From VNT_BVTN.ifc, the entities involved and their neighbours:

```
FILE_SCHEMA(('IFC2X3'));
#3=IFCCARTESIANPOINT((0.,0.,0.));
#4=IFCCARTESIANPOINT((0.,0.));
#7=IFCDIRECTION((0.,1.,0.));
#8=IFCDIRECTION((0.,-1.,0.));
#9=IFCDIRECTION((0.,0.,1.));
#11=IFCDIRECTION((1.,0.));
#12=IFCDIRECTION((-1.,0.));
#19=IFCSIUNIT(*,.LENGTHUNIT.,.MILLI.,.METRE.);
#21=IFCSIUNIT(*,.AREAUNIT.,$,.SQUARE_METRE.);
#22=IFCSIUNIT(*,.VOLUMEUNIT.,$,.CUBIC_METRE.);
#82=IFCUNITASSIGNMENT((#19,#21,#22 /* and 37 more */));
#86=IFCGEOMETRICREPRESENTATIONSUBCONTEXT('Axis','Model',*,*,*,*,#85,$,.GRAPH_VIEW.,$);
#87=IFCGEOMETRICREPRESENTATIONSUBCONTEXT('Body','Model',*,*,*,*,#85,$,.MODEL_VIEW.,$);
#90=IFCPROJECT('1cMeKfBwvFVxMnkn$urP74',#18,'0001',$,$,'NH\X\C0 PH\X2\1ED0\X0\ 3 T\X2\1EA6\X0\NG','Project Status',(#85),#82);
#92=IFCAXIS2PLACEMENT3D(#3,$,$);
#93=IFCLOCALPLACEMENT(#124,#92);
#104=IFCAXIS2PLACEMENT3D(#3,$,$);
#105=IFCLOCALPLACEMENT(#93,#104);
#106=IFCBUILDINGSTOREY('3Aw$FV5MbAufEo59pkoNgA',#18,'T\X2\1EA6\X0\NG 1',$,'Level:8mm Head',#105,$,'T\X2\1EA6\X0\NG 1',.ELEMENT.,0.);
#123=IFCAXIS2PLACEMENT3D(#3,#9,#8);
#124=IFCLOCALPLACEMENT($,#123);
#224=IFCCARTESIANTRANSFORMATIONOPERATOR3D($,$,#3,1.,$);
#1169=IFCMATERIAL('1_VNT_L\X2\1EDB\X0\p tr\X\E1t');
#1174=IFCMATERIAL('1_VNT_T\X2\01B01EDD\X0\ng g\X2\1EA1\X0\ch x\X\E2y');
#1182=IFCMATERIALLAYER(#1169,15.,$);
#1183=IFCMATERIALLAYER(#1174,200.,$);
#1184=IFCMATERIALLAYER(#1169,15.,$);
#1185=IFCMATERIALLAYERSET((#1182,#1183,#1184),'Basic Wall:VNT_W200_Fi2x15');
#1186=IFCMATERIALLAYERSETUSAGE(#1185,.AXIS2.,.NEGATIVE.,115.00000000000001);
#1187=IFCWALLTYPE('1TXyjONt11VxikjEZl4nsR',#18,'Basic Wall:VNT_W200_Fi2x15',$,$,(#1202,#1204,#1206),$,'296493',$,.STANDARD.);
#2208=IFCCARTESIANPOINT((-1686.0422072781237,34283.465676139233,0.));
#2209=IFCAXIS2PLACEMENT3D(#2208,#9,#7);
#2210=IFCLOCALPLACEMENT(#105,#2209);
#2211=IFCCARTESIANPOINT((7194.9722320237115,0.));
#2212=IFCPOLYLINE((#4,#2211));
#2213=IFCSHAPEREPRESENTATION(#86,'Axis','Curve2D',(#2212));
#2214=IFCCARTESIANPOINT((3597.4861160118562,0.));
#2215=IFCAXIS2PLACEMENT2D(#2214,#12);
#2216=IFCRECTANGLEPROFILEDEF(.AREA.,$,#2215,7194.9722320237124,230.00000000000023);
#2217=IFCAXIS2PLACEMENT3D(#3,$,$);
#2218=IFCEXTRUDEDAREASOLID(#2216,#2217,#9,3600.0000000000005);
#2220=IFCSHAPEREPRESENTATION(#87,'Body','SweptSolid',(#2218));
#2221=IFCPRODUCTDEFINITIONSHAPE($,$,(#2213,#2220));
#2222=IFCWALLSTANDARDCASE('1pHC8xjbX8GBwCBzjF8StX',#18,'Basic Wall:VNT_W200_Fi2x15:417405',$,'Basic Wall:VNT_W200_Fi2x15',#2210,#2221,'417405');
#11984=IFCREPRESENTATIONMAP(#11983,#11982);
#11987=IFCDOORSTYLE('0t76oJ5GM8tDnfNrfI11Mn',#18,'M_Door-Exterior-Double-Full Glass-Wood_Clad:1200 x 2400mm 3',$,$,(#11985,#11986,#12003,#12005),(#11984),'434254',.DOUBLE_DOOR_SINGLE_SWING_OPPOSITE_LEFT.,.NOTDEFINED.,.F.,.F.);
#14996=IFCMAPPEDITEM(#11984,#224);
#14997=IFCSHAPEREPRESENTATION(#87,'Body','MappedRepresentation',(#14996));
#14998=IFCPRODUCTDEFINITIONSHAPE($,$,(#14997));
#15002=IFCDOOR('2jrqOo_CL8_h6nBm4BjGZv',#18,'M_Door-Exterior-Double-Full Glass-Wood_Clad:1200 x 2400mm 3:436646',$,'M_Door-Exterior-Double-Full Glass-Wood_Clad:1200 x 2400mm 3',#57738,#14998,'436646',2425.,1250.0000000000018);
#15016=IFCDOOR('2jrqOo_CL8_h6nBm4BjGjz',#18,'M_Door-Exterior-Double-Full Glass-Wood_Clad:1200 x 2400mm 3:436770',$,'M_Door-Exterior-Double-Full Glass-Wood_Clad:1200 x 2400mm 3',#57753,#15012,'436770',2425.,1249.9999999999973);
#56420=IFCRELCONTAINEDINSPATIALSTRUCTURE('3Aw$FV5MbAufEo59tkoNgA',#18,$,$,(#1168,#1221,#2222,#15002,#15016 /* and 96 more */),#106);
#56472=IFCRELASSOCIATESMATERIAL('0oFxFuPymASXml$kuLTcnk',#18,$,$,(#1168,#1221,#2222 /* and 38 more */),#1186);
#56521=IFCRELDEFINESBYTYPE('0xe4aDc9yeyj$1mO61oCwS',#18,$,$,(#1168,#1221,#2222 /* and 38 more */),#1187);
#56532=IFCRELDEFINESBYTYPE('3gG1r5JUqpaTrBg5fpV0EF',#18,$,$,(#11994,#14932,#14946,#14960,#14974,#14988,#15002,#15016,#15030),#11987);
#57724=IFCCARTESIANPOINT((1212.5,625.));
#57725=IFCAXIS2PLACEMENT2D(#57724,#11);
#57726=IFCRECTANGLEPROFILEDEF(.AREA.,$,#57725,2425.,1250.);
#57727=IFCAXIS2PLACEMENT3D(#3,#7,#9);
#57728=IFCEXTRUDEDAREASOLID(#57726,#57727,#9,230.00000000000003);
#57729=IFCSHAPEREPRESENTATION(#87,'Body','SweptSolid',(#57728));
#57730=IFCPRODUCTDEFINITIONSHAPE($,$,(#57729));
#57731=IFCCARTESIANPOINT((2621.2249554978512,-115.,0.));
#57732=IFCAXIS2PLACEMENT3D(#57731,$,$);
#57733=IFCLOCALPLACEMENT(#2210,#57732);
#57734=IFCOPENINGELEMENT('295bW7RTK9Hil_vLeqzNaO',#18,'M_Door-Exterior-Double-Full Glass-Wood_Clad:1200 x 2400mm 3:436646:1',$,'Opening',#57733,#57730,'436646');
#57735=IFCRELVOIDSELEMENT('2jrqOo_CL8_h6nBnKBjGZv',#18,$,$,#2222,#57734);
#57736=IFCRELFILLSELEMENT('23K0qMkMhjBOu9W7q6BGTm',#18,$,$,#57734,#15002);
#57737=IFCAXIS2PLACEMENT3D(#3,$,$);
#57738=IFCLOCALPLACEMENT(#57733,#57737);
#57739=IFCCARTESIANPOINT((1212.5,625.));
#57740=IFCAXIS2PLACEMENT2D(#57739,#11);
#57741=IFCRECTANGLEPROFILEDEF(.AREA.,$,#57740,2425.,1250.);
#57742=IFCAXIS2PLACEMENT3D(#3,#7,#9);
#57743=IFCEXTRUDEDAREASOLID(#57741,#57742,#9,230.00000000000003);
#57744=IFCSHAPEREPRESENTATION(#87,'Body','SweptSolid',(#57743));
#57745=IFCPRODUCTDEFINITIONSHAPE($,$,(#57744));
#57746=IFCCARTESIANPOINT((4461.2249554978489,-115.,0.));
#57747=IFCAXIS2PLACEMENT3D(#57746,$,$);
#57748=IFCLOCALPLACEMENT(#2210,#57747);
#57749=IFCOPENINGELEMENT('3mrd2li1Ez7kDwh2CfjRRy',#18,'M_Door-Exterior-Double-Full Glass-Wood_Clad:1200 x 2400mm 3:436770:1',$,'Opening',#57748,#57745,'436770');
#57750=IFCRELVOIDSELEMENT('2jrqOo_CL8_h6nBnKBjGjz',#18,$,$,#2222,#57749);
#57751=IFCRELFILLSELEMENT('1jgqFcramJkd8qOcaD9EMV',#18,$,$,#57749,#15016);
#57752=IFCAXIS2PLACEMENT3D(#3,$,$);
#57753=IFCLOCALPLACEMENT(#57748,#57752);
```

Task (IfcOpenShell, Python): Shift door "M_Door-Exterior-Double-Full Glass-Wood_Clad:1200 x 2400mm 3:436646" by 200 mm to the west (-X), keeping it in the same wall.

```python
import ifcopenshell
import ifcopenshell.api.geometry
import ifcopenshell.util.placement

model = ifcopenshell.open("VNT_BVTN.ifc")

door = model.by_guid("2jrqOo_CL8_h6nBm4BjGZv")
opening = door.FillsVoids[0].RelatingOpeningElement
wall = opening.VoidsElements[0].RelatingBuildingElement

wall_matrix = ifcopenshell.util.placement.get_local_placement(wall.ObjectPlacement)
shift = wall_matrix[:3, 0] * -200.0
before = ifcopenshell.util.placement.get_local_placement(door.ObjectPlacement)[:3, 3].copy()

# The door is placed relative to its opening, so it follows when the opening moves.
matrix = ifcopenshell.util.placement.get_local_placement(opening.ObjectPlacement)
matrix[:3, 3] += shift
ifcopenshell.api.geometry.edit_object_placement(
    model, product=opening, matrix=matrix, is_si=False, should_transform_children=True
)

after = ifcopenshell.util.placement.get_local_placement(door.ObjectPlacement)[:3, 3]
print("door moved by", (after - before).round(3) + 0.0)

model.write("VNT_BVTN_edited.ifc")
```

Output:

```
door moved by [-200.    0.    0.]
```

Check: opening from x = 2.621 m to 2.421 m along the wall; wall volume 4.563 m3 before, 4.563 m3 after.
